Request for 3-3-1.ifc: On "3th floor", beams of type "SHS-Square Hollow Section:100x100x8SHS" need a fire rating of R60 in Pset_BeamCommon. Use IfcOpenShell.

First a look at what the model holds.

```python
import ifcopenshell
import ifcopenshell.util.element

model = ifcopenshell.open("3-3-1.ifc")
print(model.schema)
storey = next(s for s in model.by_type("IfcBuildingStorey") if s.Name == "3th floor")
beams = [e for e in ifcopenshell.util.element.get_decomposition(storey) if e.is_a("IfcBeam")]
seen = {}
for e in beams:
    element_type = ifcopenshell.util.element.get_type(e)
    key = (element_type.Name if element_type != e and element_type else None, ifcopenshell.util.element.get_pset(e, "Pset_BeamCommon", "FireRating"))
    seen[key] = seen.get(key, 0) + 1
for (name, value), count in sorted(seen.items(), key=str):
    print(count, "x", name, "|", value)
```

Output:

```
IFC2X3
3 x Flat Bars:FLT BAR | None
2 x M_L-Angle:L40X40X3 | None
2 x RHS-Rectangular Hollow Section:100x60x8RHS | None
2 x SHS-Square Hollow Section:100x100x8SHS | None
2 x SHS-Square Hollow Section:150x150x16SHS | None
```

```python
import ifcopenshell
import ifcopenshell.api.pset
import ifcopenshell.util.element

model = ifcopenshell.open("3-3-1.ifc")

storey = next(s for s in model.by_type("IfcBuildingStorey") if s.Name == "3th floor")
beams = [e for e in ifcopenshell.util.element.get_decomposition(storey) if e.is_a("IfcBeam")]

count = 0
for e in beams:
    element_type = ifcopenshell.util.element.get_type(e)
    if element_type in (None, e) or element_type.Name != "SHS-Square Hollow Section:100x100x8SHS":
        continue
    # add_pset returns the element's existing set when there is one.
    pset = ifcopenshell.api.pset.add_pset(model, product=e, name="Pset_BeamCommon")
    ifcopenshell.api.pset.edit_pset(model, pset=pset, properties={"FireRating": "R60"})
    count += 1

print(count, "beams updated")

model.write("3-3-1-out.ifc")
```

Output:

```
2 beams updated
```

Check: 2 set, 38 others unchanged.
